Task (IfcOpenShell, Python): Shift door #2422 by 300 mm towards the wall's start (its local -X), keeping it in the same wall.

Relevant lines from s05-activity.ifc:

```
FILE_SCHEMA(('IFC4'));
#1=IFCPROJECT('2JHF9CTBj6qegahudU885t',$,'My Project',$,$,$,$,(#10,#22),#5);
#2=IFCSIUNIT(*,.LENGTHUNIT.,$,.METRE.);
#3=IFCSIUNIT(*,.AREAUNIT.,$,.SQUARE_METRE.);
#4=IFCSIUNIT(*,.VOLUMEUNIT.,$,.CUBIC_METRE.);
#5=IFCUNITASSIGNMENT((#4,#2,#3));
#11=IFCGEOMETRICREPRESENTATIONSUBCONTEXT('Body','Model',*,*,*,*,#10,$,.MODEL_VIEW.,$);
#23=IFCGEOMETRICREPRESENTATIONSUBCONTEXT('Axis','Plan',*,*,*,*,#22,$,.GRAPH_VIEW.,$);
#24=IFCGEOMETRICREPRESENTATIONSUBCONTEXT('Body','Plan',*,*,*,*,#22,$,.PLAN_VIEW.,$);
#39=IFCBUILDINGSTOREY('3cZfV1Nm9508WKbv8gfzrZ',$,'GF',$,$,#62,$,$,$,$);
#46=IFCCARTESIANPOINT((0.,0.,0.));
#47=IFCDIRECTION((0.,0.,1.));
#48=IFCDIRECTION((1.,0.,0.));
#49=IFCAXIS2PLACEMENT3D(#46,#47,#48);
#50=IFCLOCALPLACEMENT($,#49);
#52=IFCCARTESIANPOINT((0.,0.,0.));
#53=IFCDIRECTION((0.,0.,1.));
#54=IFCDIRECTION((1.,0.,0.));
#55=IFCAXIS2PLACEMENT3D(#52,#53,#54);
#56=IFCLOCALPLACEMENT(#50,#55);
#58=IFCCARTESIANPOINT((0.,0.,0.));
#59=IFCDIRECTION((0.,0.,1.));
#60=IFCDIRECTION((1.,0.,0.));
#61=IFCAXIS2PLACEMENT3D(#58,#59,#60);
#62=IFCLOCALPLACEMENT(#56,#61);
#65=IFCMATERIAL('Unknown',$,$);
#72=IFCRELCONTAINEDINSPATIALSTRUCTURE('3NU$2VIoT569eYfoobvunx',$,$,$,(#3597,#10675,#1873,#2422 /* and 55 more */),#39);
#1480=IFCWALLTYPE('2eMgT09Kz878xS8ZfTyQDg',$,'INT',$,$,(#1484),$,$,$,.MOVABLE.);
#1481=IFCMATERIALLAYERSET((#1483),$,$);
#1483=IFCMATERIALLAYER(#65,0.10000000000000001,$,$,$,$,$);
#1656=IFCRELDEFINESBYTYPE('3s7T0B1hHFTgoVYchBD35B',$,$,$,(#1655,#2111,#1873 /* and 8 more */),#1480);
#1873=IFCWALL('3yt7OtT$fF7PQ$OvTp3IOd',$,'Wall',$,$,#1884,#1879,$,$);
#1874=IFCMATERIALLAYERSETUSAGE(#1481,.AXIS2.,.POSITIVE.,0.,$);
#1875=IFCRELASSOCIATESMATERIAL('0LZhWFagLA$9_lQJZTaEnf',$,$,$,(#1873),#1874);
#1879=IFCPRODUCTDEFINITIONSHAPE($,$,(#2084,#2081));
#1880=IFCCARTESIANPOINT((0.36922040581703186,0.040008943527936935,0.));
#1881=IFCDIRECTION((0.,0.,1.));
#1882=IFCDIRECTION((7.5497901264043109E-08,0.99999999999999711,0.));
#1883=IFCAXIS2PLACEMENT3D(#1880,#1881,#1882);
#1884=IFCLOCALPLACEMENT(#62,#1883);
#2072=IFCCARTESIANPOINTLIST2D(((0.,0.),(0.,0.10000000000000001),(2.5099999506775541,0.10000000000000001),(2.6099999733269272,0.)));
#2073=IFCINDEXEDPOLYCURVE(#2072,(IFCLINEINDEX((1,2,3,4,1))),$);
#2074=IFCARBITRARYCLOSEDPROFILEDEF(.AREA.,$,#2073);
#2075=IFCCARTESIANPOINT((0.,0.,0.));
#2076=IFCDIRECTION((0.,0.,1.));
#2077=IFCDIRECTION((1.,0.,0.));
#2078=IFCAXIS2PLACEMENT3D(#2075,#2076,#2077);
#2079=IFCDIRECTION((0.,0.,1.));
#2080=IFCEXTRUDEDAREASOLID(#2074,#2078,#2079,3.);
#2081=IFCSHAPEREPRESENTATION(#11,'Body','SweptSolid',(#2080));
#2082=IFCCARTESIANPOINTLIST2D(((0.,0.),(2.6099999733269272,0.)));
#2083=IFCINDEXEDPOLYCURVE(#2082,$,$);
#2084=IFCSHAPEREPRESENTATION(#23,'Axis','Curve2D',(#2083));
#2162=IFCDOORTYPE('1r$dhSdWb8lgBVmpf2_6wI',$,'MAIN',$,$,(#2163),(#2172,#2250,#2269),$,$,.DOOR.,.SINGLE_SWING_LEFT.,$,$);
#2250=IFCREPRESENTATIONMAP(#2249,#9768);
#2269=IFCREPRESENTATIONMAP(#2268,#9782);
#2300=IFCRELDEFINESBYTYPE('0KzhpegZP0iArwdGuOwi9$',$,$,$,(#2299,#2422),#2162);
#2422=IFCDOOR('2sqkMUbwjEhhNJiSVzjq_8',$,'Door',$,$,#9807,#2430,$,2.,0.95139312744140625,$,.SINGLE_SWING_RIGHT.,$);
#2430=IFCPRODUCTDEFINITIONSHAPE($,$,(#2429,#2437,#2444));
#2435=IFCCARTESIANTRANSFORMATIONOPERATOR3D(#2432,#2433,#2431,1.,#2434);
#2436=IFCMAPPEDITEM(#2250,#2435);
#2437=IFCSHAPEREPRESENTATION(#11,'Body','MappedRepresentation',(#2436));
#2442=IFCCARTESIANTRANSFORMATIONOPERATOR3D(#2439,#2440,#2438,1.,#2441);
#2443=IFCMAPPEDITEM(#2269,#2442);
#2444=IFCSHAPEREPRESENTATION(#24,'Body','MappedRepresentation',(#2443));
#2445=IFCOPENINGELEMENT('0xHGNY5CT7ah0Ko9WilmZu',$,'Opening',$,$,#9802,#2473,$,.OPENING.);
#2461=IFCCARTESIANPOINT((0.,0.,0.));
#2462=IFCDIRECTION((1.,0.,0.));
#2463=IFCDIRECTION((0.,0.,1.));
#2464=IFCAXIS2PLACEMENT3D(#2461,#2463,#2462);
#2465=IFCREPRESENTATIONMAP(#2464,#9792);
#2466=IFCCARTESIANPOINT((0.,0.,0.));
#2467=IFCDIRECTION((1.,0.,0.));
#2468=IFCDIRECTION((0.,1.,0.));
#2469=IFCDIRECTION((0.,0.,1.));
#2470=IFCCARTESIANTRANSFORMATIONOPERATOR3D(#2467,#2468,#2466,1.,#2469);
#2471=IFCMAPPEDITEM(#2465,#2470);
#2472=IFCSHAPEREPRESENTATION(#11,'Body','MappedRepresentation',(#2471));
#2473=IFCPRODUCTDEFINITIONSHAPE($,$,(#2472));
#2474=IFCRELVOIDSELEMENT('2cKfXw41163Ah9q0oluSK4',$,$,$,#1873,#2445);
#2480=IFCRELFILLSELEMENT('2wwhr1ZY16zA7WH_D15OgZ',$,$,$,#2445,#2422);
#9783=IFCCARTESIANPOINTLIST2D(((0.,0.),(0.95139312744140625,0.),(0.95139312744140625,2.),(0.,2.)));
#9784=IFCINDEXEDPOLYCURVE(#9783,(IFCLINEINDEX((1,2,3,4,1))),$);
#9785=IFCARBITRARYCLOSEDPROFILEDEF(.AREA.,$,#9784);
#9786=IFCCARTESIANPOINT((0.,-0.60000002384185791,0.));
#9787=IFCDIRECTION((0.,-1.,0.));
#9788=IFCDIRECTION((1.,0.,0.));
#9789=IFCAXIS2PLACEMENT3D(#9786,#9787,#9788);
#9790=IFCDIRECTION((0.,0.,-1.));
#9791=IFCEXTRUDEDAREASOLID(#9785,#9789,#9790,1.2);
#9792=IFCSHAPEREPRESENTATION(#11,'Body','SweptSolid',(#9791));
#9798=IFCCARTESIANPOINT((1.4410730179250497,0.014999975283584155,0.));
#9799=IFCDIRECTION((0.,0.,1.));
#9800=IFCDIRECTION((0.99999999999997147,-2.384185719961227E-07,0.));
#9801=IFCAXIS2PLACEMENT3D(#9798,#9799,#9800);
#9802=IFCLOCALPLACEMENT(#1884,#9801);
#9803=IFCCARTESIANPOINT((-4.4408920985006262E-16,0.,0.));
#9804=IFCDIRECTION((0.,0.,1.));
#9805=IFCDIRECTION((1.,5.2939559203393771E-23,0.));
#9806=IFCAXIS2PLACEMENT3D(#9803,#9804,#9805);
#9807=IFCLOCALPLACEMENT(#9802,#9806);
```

```python
import ifcopenshell
import ifcopenshell.api.geometry
import ifcopenshell.util.placement
import ifcopenshell.util.unit

model = ifcopenshell.open("s05-activity.ifc")
unit_scale = ifcopenshell.util.unit.calculate_unit_scale(model)

door = model.by_guid("2sqkMUbwjEhhNJiSVzjq_8")
opening = door.FillsVoids[0].RelatingOpeningElement
wall = opening.VoidsElements[0].RelatingBuildingElement

wall_matrix = ifcopenshell.util.placement.get_local_placement(wall.ObjectPlacement)
shift = wall_matrix[:3, 0] * -0.3 / unit_scale
before = ifcopenshell.util.placement.get_local_placement(door.ObjectPlacement)[:3, 3].copy()

# The door is placed relative to its opening, so it follows when the opening moves.
matrix = ifcopenshell.util.placement.get_local_placement(opening.ObjectPlacement)
matrix[:3, 3] += shift
ifcopenshell.api.geometry.edit_object_placement(
    model, product=opening, matrix=matrix, is_si=False, should_transform_children=True
)

after = ifcopenshell.util.placement.get_local_placement(door.ObjectPlacement)[:3, 3]
print("door moved by", (after - before).round(3) + 0.0)

model.write("s05-activity_updated.ifc")
```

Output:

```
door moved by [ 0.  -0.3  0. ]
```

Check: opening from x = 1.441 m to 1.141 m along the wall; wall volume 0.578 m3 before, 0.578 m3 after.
